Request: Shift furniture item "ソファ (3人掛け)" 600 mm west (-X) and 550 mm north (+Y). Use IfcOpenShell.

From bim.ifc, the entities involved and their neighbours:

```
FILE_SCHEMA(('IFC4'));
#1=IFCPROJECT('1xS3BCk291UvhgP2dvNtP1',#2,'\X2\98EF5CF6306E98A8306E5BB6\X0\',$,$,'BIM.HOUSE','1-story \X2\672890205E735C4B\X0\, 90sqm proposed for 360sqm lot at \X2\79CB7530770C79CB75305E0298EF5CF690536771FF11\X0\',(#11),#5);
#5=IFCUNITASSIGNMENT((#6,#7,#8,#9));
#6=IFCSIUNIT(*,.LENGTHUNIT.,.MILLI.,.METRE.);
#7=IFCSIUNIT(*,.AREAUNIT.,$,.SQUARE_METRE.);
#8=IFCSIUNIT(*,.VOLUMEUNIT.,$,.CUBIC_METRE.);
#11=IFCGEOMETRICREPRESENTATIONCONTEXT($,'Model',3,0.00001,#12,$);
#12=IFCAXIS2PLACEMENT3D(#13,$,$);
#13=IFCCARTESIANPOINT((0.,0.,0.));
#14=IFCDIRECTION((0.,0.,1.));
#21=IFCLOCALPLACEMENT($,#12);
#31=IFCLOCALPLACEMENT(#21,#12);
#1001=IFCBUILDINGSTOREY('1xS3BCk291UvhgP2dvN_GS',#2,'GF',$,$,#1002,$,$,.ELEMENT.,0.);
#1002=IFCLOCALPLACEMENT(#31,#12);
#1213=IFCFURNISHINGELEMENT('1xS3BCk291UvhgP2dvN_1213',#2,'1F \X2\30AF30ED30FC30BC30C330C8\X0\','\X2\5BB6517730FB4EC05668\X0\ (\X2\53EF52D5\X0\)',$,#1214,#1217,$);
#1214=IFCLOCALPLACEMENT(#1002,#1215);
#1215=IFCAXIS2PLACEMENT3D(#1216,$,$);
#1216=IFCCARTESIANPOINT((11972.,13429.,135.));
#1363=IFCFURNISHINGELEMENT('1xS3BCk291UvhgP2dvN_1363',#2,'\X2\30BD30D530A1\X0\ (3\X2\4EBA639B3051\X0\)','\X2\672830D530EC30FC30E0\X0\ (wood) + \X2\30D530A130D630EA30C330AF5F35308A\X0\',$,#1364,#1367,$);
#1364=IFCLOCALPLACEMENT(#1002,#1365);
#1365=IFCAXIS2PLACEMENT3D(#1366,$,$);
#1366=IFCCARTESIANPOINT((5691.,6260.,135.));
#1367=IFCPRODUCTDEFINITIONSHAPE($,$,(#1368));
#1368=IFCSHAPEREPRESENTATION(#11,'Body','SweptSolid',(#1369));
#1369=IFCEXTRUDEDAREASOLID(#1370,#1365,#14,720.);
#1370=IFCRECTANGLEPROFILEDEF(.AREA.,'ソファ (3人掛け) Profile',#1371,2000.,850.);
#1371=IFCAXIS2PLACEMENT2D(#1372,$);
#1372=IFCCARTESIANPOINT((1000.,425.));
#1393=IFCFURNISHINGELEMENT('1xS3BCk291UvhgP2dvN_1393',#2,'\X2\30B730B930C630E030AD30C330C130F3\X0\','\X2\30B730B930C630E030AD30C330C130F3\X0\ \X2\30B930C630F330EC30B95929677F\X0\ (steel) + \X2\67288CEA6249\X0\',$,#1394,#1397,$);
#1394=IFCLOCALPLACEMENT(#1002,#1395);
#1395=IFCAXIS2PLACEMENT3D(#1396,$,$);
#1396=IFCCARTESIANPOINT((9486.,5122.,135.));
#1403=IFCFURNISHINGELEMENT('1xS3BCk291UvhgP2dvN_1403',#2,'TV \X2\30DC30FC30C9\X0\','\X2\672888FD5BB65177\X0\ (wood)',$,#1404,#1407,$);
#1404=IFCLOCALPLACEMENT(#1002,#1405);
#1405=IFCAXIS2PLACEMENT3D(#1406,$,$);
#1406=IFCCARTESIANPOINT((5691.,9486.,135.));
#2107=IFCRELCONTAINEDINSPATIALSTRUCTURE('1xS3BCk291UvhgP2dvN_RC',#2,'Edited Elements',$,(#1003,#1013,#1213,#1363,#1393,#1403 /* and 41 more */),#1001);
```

```python
import ifcopenshell
import ifcopenshell.api.geometry
import ifcopenshell.util.placement
import ifcopenshell.util.unit

model = ifcopenshell.open("bim.ifc")
unit_scale = ifcopenshell.util.unit.calculate_unit_scale(model)

item = model.by_id(1363)
matrix = ifcopenshell.util.placement.get_local_placement(item.ObjectPlacement)
matrix[0, 3] -= 0.6 / unit_scale
matrix[1, 3] += 0.55 / unit_scale
ifcopenshell.api.geometry.edit_object_placement(model, product=item, matrix=matrix, is_si=False)

print(ifcopenshell.util.placement.get_local_placement(item.ObjectPlacement).round(3) + 0.0)

model.write("bim_updated.ifc")
```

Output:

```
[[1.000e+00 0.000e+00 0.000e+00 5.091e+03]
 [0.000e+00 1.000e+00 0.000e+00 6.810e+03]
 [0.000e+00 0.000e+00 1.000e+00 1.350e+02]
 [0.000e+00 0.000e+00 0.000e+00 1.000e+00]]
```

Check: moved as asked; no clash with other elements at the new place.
